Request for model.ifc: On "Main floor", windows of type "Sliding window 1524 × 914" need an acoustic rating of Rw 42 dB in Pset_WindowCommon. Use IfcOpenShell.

First a look at what the model holds.

```python
import ifcopenshell
import ifcopenshell.util.element

model = ifcopenshell.open("model.ifc")
print(model.schema)
storey = next(s for s in model.by_type("IfcBuildingStorey") if s.Name == "Main floor")
windows = [e for e in ifcopenshell.util.element.get_decomposition(storey) if e.is_a("IfcWindow")]
seen = {}
for e in windows:
    element_type = ifcopenshell.util.element.get_type(e)
    key = (element_type.Name if element_type != e and element_type else None, ifcopenshell.util.element.get_pset(e, "Pset_WindowCommon", "AcousticRating"))
    seen[key] = seen.get(key, 0) + 1
for (name, value), count in sorted(seen.items(), key=str):
    print(count, "x", name, "|", value)
```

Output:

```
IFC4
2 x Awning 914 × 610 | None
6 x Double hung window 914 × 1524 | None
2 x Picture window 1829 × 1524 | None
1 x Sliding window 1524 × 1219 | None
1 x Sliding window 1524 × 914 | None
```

```python
import ifcopenshell
import ifcopenshell.api.pset
import ifcopenshell.util.element

model = ifcopenshell.open("model.ifc")

storey = next(s for s in model.by_type("IfcBuildingStorey") if s.Name == "Main floor")
windows = [e for e in ifcopenshell.util.element.get_decomposition(storey) if e.is_a("IfcWindow")]

count = 0
for e in windows:
    element_type = ifcopenshell.util.element.get_type(e)
    if element_type in (None, e) or element_type.Name != "Sliding window 1524 × 914":
        continue
    # add_pset returns the element's existing set when there is one.
    pset = ifcopenshell.api.pset.add_pset(model, product=e, name="Pset_WindowCommon")
    ifcopenshell.api.pset.edit_pset(model, pset=pset, properties={"AcousticRating": "Rw 42 dB"})
    count += 1

print(count, "windows updated")

model.write("model_updated.ifc")
```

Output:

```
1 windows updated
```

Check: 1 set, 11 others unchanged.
